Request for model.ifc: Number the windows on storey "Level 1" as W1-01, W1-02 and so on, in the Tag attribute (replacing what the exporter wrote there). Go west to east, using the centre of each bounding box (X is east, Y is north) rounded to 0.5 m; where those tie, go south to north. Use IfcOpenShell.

First a look at what the model holds.

```python
import ifcopenshell
import ifcopenshell.util.element
import ifcopenshell.util.placement

model = ifcopenshell.open("model.ifc")
print(model.schema)
storey = next(s for s in model.by_type("IfcBuildingStorey") if s.Name == "Level 1")
windows = [e for e in ifcopenshell.util.element.get_decomposition(storey) if e.is_a("IfcWindow")]
for e in sorted(windows, key=lambda e: e.id()):
    origin = ifcopenshell.util.placement.get_local_placement(e.ObjectPlacement)[:3, 3]
    print(e.id(), e.Tag, e.Name, origin.round(2) + 0.0, sep=" | ")
```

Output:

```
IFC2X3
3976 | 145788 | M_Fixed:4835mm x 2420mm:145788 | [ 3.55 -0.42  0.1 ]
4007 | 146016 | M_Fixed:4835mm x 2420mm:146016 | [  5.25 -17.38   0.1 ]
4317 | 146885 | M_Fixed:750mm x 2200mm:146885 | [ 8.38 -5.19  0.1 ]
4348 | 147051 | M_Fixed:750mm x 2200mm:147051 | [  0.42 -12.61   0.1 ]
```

```python
import ifcopenshell
import ifcopenshell.geom
import ifcopenshell.util.element
import ifcopenshell.util.shape

model = ifcopenshell.open("model.ifc")
settings = ifcopenshell.geom.settings()
settings.set("use-world-coords", True)


def centre(element):
    shape = ifcopenshell.geom.create_shape(settings, element)
    return ifcopenshell.util.shape.get_bbox_centroid(shape.geometry)


storey = next(s for s in model.by_type("IfcBuildingStorey") if s.Name == "Level 1")
windows = [e for e in ifcopenshell.util.element.get_decomposition(storey) if e.is_a("IfcWindow")]

# Insertion points can sit at a corner or the storey origin, so sort by the geometry (in metres).
centres = {e: centre(e) for e in windows}
windows.sort(key=lambda e: (round(centres[e][0] / 0.5), centres[e][1]))

for i, e in enumerate(windows, start=1):
    number = f"W1-{i:02d}"
    e.Tag = number
    print(e.id(), number)

model.write("model_updated.ifc")
```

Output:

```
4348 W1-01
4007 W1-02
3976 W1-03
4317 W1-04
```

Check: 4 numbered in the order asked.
